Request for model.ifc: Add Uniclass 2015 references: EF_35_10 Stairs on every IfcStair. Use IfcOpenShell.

First a look at what the model holds.

```python
import ifcopenshell

model = ifcopenshell.open("model.ifc")
print(model.schema)
print("classifications:", [c.Name for c in model.by_type("IfcClassification")])
for ifc_class in ("IfcDoor", "IfcRoof", "IfcStair", "IfcWall", "IfcWindow"):
    print(ifc_class, len(model.by_type(ifc_class)))
```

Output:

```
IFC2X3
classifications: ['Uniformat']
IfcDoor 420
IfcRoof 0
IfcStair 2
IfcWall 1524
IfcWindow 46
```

```python
import ifcopenshell
import ifcopenshell.api.classification

model = ifcopenshell.open("model.ifc")

# IFC2X3 requires Source and Edition and has no link from the project to the system.
system = model.create_entity("IfcClassification", Source="NBS", Edition="2015", Name="Uniclass 2015")

codes = {
    "IfcStair": ("EF_35_10", "Stairs"),
}
for ifc_class, (code, name) in codes.items():
    products = model.by_type(ifc_class)
    ifcopenshell.api.classification.add_reference(
        model, products=products, classification=system, identification=code, name=name
    )
    print(code, len(products))

model.write("model_updated.ifc")
```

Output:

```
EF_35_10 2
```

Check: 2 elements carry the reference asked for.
